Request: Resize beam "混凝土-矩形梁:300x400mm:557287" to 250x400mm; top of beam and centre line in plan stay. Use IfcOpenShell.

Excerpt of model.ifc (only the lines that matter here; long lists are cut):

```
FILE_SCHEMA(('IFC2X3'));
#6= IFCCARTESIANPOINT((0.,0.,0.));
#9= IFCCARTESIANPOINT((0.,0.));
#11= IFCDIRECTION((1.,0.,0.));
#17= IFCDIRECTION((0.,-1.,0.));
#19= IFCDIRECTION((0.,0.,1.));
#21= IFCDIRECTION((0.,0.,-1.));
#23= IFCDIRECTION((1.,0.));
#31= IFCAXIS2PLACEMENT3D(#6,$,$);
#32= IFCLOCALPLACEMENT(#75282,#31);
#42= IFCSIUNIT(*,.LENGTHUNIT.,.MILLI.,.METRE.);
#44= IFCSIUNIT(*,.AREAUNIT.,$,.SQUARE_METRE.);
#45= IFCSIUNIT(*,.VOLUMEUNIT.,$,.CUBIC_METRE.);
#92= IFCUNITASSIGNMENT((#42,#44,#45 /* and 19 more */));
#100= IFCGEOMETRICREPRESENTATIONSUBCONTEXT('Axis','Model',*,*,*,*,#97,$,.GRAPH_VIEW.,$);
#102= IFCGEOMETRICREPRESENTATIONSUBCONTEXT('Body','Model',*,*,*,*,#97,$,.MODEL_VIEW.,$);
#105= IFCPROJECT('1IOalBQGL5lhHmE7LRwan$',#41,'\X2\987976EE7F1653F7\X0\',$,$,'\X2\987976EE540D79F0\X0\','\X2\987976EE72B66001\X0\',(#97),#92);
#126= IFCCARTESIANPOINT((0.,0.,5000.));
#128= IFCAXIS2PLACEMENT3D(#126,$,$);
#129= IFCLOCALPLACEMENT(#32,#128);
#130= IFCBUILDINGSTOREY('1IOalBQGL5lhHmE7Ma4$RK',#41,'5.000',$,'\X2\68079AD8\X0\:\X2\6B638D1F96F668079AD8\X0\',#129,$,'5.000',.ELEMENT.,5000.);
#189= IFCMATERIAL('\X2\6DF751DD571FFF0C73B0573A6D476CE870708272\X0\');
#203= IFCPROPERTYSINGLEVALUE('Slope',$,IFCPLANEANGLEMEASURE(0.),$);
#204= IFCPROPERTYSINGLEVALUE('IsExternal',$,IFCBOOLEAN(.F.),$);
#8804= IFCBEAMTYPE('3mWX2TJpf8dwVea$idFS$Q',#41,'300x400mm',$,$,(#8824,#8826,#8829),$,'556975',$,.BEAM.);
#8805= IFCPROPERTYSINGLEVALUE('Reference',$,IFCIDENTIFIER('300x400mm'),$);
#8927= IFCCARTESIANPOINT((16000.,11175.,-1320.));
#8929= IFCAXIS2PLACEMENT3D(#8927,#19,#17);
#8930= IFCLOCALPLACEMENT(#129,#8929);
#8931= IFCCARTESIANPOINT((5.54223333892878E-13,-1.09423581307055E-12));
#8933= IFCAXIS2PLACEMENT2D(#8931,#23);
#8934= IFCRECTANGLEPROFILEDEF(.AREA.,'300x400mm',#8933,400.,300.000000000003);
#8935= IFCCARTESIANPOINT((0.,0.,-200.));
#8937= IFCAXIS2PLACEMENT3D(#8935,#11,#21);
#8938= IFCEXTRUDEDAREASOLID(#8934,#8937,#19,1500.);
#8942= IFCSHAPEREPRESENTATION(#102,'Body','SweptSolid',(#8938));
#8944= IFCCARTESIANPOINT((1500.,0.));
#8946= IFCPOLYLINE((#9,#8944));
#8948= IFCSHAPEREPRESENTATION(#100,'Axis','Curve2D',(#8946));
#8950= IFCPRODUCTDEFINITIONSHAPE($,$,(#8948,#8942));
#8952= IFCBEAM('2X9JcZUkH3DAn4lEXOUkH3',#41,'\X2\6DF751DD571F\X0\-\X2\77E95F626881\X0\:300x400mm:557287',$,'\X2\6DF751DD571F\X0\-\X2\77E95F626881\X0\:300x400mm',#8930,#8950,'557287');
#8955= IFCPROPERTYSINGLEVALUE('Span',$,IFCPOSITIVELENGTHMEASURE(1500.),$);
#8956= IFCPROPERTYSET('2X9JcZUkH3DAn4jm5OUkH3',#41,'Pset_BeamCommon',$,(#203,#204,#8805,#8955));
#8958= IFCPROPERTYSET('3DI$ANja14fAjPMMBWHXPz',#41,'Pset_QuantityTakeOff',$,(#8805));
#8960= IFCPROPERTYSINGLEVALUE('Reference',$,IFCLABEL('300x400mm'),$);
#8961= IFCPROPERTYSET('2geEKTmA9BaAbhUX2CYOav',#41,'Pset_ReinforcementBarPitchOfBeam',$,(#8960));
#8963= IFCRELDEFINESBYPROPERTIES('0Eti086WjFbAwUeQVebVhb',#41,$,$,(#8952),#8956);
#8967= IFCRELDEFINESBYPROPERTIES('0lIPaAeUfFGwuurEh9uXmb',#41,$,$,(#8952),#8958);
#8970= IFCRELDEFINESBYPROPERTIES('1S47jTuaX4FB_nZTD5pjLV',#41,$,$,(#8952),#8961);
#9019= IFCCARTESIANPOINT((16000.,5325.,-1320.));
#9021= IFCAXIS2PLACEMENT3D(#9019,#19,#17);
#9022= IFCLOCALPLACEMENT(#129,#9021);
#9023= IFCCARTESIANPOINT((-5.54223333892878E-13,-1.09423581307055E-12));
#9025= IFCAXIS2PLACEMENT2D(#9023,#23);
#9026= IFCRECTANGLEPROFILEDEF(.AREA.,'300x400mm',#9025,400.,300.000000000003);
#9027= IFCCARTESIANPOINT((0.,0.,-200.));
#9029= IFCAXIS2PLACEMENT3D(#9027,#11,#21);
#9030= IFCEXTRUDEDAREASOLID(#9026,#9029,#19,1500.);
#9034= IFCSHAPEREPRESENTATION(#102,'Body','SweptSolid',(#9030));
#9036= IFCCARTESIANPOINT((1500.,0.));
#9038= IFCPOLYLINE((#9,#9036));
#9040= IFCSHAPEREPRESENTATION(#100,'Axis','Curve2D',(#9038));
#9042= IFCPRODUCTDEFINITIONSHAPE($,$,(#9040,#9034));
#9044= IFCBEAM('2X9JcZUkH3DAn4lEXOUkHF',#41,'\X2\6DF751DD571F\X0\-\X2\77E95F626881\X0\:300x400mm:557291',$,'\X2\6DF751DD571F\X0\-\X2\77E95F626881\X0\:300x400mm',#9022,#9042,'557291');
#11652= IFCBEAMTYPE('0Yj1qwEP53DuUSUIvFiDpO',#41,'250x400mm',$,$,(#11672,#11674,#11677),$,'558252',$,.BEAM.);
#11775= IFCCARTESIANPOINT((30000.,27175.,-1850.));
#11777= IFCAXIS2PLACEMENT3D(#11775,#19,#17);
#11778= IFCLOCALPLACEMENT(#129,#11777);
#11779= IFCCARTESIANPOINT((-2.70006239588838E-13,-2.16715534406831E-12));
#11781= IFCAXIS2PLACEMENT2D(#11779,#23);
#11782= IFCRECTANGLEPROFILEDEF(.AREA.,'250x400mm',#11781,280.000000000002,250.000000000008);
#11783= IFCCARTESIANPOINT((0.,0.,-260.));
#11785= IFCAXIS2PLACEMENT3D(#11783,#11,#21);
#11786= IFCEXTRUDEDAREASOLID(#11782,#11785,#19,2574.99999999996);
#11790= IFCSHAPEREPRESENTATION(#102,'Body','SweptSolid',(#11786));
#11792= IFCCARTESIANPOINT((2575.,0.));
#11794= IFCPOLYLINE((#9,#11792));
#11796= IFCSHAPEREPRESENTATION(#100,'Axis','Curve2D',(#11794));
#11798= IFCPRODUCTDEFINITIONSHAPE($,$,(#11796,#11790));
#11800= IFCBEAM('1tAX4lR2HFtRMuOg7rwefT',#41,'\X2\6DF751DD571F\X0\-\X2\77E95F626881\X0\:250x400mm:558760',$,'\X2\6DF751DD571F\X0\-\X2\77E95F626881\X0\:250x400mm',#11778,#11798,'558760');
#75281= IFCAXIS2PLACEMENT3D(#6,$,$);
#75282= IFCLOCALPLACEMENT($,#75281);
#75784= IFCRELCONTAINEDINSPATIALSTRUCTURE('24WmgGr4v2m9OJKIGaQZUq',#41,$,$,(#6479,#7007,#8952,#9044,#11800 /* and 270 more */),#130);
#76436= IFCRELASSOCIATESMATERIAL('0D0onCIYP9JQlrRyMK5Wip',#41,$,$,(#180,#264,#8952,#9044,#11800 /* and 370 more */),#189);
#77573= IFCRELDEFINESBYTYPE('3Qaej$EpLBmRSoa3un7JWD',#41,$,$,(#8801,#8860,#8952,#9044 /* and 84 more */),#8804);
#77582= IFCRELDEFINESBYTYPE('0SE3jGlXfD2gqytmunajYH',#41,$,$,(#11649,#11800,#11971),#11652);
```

```python
import ifcopenshell
import ifcopenshell.api.pset
import ifcopenshell.api.type
import ifcopenshell.util.element
import ifcopenshell.util.representation

model = ifcopenshell.open("model.ifc")

member = model.by_guid("2X9JcZUkH3DAn4lEXOUkH3")
source = next(p for p in model.by_type("IfcRectangleProfileDef") if p.ProfileName == "250x400mm")

body = ifcopenshell.util.representation.get_representation(member, "Model", "Body")
solid = body.Items[0]
old_profile = solid.SweptArea

# Copy the section's sizes but keep this member's own profile position.
profile = ifcopenshell.util.element.copy(model, source)
# Profiles are centred, so shift by half the change in depth to hold the top.
shift = (old_profile.XDim - profile.XDim) / 2
x, y = old_profile.Position.Location.Coordinates
up = (-1.0, 0.0)  # upwards, in the solid's own plane
location = model.createIfcCartesianPoint((x + up[0] * shift, y + up[1] * shift))
profile.Position = model.createIfcAxis2Placement2D(location, old_profile.Position.RefDirection)
solid.SweptArea = profile
if not model.get_total_inverses(old_profile):
    ifcopenshell.util.element.remove_deep2(model, old_profile)

new_type = model.by_guid("0Yj1qwEP53DuUSUIvFiDpO")
ifcopenshell.api.type.assign_type(
    model, related_objects=[member], relating_type=new_type, should_map_representations=False
)
member.Name = member.Name.replace("300x400mm", "250x400mm")
member.ObjectType = "混凝土-矩形梁:250x400mm"
pset = model.by_id(ifcopenshell.util.element.get_pset(member, "Pset_BeamCommon", should_inherit=False)["id"])
ifcopenshell.api.pset.edit_pset(model, pset=pset, properties={"Reference": "250x400mm"})
pset = model.by_id(ifcopenshell.util.element.get_pset(member, "Pset_QuantityTakeOff", should_inherit=False)["id"])
ifcopenshell.api.pset.edit_pset(model, pset=pset, properties={"Reference": "250x400mm"})
pset = model.by_id(ifcopenshell.util.element.get_pset(member, "Pset_ReinforcementBarPitchOfBeam", should_inherit=False)["id"])
ifcopenshell.api.pset.edit_pset(model, pset=pset, properties={"Reference": "250x400mm"})

print(solid.SweptArea)

model.write("model_updated.ifc")
```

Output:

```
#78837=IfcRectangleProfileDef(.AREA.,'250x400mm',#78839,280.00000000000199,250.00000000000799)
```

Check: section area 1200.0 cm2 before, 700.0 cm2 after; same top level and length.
